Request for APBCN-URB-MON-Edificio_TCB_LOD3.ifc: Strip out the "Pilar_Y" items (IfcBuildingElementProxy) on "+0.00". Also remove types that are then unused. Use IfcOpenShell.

First a look at what the model holds.

```python
import ifcopenshell
import ifcopenshell.util.element

model = ifcopenshell.open("APBCN-URB-MON-Edificio_TCB_LOD3.ifc")
print(model.schema)
storey = next(s for s in model.by_type("IfcBuildingStorey") if s.Name == "+0.00")
proxies = [e for e in ifcopenshell.util.element.get_decomposition(storey) if e.is_a("IfcBuildingElementProxy")]
seen = {}
for e in proxies:
    element_type = ifcopenshell.util.element.get_type(e)
    name = element_type.Name if element_type not in (None, e) else None
    seen[name] = seen.get(name, 0) + 1
for name, count in sorted(seen.items(), key=str):
    print(count, "x", name)
```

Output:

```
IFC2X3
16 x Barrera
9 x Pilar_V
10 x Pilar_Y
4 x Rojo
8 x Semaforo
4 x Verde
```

```python
import ifcopenshell
import ifcopenshell.api.root
import ifcopenshell.util.element

model = ifcopenshell.open("APBCN-URB-MON-Edificio_TCB_LOD3.ifc")

storey = next(s for s in model.by_type("IfcBuildingStorey") if s.Name == "+0.00")
proxies = [e for e in ifcopenshell.util.element.get_decomposition(storey) if e.is_a("IfcBuildingElementProxy")]
targets = [e for e in proxies if (t := ifcopenshell.util.element.get_type(e)) not in (None, e) and t.Name == "Pilar_Y"]
types = {ifcopenshell.util.element.get_type(e) for e in targets} - {None, *targets}

for e in targets:
    ifcopenshell.api.root.remove_product(model, product=e)
print(len(targets), "removed")

unused = [t for t in types if not ifcopenshell.util.element.get_types(t)]
for t in unused:
    ifcopenshell.api.root.remove_product(model, product=t)
print(len(unused), "unused types removed")

model.write("APBCN-URB-MON-Edificio_TCB_LOD3_updated.ifc")
```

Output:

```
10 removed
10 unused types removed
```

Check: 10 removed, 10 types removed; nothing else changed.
